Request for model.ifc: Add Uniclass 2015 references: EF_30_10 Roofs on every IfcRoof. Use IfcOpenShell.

First a look at what the model holds.

```python
import ifcopenshell

model = ifcopenshell.open("model.ifc")
print(model.schema)
print("classifications:", [c.Name for c in model.by_type("IfcClassification")])
for ifc_class in ("IfcDoor", "IfcRoof", "IfcStair", "IfcWall", "IfcWindow"):
    print(ifc_class, len(model.by_type(ifc_class)))
```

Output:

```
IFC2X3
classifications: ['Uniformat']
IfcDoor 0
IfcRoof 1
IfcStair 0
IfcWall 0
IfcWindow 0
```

```python
import ifcopenshell
import ifcopenshell.api.classification

model = ifcopenshell.open("model.ifc")

# IFC2X3 requires Source and Edition and has no link from the project to the system.
system = model.create_entity("IfcClassification", Source="NBS", Edition="2015", Name="Uniclass 2015")

codes = {
    "IfcRoof": ("EF_30_10", "Roofs"),
}
for ifc_class, (code, name) in codes.items():
    products = model.by_type(ifc_class)
    ifcopenshell.api.classification.add_reference(
        model, products=products, classification=system, identification=code, name=name
    )
    print(code, len(products))

model.write("model_rev.ifc")
```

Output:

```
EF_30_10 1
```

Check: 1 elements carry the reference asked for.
